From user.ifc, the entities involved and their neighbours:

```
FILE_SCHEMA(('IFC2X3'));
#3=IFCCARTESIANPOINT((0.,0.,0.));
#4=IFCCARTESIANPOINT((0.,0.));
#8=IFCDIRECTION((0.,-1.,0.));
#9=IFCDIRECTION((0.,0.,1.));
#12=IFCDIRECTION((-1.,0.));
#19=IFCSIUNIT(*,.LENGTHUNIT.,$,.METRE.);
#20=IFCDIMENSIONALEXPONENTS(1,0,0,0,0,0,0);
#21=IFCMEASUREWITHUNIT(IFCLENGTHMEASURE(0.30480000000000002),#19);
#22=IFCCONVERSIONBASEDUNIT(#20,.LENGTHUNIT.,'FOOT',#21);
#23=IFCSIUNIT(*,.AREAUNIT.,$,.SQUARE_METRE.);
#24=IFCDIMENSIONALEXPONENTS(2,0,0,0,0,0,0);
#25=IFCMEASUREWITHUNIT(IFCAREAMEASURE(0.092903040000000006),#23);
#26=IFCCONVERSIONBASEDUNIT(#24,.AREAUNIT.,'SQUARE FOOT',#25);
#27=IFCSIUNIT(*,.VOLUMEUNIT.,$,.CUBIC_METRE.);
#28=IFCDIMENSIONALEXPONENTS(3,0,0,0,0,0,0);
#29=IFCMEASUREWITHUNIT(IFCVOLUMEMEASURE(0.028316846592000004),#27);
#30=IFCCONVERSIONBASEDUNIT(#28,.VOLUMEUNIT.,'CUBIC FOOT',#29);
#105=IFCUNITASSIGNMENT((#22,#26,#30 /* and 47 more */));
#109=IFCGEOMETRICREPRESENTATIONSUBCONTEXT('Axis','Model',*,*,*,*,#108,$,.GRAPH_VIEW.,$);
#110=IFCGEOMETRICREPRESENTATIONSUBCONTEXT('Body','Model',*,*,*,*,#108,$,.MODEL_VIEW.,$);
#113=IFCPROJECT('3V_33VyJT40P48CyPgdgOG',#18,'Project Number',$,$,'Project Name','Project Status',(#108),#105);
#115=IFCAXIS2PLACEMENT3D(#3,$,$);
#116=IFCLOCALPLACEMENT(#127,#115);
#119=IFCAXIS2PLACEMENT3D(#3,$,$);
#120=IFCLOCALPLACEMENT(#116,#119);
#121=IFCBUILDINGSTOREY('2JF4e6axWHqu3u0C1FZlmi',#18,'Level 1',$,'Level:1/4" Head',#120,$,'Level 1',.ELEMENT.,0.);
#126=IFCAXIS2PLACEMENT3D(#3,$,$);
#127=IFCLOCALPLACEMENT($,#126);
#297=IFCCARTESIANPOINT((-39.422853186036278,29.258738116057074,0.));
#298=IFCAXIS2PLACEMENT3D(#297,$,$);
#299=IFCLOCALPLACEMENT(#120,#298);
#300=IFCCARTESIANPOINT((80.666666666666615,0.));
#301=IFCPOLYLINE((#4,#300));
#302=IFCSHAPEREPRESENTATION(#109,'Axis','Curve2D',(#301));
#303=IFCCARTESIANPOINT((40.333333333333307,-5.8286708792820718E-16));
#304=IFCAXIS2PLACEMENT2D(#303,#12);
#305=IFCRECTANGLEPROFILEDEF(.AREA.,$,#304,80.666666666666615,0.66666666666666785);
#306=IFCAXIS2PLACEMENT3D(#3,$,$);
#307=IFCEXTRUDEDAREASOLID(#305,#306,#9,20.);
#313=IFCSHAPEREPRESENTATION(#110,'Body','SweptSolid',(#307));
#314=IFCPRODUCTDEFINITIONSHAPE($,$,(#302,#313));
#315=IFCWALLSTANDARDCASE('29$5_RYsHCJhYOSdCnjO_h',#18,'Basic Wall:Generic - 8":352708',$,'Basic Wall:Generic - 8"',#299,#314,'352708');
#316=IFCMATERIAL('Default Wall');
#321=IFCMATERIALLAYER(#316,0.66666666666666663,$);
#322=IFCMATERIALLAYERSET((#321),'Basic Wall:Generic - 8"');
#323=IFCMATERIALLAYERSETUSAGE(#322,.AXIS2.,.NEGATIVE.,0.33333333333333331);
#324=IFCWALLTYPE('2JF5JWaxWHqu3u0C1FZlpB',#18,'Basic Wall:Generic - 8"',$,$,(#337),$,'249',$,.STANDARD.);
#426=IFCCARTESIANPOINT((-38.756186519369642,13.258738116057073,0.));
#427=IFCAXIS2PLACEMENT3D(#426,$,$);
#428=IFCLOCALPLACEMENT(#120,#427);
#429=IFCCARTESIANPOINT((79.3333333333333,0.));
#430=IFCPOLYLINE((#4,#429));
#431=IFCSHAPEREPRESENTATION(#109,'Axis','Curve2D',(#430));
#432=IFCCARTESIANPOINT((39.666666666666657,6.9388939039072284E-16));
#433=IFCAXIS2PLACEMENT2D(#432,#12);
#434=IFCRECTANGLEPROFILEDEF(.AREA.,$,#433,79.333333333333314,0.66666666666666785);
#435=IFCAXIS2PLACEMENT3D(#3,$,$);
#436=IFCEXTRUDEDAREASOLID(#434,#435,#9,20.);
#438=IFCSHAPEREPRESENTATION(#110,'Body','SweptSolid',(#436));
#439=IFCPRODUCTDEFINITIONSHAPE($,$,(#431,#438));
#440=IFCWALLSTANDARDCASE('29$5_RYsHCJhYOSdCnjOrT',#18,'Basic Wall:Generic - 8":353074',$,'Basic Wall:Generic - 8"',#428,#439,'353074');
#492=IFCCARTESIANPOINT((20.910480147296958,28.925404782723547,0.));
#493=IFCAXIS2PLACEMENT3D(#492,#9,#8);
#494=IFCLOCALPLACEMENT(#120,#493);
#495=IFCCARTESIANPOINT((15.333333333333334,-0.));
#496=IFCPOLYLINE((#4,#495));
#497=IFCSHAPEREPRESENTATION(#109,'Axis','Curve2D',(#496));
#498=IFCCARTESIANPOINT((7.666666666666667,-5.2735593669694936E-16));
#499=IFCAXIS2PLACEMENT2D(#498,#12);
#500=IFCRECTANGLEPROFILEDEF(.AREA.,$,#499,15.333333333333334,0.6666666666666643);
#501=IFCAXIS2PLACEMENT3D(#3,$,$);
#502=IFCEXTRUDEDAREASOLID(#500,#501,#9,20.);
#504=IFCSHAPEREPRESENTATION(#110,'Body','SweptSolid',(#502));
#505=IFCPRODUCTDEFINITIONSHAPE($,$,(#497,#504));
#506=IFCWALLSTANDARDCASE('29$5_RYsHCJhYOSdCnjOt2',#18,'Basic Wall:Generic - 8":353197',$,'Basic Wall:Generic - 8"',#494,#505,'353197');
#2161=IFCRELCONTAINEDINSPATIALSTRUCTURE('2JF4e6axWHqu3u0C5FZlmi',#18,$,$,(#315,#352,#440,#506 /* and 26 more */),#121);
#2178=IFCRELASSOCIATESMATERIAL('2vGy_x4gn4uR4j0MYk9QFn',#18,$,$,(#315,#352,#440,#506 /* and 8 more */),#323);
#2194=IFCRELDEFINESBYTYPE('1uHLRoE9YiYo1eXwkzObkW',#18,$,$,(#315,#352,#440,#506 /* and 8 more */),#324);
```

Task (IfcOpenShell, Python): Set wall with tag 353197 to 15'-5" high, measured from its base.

```python
import ifcopenshell
import ifcopenshell.geom
import ifcopenshell.util.representation
import ifcopenshell.util.shape
import ifcopenshell.util.unit

model = ifcopenshell.open("user.ifc")
unit_scale = ifcopenshell.util.unit.calculate_unit_scale(model)
settings = ifcopenshell.geom.settings()


def volume(element):
    """Net volume in cubic metres, openings subtracted."""
    shape = ifcopenshell.geom.create_shape(settings, element)
    return ifcopenshell.util.shape.get_volume(shape.geometry)


wall = model.by_guid("29$5_RYsHCJhYOSdCnjOt2")
before = volume(wall)

body = ifcopenshell.util.representation.get_representation(wall, "Model", "Body")
solid = body.Items[0]
old_height = solid.Depth
solid.Depth = 185 * 0.0254 / unit_scale
after = volume(wall)

print(f"height {old_height:g} -> {solid.Depth:g}, volume {before:.3f} -> {after:.3f} m3")

model.write("user_v2.ifc")
```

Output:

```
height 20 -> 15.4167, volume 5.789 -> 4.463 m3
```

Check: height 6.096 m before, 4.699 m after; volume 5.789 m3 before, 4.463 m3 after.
